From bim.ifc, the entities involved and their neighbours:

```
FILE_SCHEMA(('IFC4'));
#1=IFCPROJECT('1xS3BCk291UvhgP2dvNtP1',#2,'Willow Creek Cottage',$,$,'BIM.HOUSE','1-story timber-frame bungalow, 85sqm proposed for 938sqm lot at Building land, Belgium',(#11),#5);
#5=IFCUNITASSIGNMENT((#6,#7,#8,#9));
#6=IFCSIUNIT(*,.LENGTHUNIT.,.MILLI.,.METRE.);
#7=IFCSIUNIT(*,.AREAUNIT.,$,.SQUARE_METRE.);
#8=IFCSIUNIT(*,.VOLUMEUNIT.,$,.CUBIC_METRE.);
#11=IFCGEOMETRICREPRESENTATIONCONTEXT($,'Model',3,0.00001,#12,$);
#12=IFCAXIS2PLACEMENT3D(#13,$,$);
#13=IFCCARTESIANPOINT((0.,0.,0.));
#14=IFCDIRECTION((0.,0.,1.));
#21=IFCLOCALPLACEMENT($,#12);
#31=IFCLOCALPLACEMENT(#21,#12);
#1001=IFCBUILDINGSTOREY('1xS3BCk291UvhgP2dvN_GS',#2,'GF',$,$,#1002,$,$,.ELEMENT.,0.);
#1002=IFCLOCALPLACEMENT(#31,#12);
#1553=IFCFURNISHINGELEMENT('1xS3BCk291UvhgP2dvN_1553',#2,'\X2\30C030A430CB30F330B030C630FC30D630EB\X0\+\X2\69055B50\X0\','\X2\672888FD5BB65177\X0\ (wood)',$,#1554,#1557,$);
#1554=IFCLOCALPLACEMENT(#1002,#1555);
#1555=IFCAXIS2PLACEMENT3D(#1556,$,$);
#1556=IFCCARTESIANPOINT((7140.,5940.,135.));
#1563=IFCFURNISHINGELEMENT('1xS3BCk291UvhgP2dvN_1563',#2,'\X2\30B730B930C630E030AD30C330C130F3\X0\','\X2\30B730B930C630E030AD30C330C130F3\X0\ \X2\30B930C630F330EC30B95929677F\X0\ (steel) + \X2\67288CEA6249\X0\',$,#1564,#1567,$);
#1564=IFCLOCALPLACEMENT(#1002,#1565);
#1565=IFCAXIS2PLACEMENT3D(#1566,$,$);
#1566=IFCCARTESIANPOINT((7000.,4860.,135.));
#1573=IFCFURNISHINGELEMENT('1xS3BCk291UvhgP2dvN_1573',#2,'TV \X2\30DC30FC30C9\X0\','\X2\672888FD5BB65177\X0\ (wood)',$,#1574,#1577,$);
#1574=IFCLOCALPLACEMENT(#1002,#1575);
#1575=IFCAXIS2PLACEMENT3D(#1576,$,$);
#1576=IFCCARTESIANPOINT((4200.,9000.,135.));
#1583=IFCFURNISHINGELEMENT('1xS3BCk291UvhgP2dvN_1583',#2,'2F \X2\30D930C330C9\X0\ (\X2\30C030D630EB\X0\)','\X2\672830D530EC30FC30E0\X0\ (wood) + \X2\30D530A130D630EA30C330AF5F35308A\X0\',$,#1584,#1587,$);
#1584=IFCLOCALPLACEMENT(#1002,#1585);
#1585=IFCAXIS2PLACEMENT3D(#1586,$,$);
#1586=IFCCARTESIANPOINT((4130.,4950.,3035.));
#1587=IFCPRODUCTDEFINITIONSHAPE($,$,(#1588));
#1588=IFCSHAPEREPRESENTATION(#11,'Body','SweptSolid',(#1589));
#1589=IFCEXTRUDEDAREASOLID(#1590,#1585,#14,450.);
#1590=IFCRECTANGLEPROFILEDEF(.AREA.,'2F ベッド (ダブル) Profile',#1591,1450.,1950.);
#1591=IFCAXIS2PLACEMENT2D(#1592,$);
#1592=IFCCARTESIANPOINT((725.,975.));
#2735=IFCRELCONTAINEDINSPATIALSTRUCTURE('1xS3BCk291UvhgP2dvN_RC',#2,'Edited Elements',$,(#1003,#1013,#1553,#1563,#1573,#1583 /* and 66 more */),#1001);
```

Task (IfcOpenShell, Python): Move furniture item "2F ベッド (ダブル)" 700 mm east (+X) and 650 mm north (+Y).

```python
import ifcopenshell
import ifcopenshell.api.geometry
import ifcopenshell.util.placement

model = ifcopenshell.open("bim.ifc")

item = model.by_guid("1xS3BCk291UvhgP2dvN_1583")
matrix = ifcopenshell.util.placement.get_local_placement(item.ObjectPlacement)
matrix[0, 3] += 700.0
matrix[1, 3] += 650.0
ifcopenshell.api.geometry.edit_object_placement(model, product=item, matrix=matrix, is_si=False)

print(ifcopenshell.util.placement.get_local_placement(item.ObjectPlacement).round(3) + 0.0)

model.write("bim-out.ifc")
```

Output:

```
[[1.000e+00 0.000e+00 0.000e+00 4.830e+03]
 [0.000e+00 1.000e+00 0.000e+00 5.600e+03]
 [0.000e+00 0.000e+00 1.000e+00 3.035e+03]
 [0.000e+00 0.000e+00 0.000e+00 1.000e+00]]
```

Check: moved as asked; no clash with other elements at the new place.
